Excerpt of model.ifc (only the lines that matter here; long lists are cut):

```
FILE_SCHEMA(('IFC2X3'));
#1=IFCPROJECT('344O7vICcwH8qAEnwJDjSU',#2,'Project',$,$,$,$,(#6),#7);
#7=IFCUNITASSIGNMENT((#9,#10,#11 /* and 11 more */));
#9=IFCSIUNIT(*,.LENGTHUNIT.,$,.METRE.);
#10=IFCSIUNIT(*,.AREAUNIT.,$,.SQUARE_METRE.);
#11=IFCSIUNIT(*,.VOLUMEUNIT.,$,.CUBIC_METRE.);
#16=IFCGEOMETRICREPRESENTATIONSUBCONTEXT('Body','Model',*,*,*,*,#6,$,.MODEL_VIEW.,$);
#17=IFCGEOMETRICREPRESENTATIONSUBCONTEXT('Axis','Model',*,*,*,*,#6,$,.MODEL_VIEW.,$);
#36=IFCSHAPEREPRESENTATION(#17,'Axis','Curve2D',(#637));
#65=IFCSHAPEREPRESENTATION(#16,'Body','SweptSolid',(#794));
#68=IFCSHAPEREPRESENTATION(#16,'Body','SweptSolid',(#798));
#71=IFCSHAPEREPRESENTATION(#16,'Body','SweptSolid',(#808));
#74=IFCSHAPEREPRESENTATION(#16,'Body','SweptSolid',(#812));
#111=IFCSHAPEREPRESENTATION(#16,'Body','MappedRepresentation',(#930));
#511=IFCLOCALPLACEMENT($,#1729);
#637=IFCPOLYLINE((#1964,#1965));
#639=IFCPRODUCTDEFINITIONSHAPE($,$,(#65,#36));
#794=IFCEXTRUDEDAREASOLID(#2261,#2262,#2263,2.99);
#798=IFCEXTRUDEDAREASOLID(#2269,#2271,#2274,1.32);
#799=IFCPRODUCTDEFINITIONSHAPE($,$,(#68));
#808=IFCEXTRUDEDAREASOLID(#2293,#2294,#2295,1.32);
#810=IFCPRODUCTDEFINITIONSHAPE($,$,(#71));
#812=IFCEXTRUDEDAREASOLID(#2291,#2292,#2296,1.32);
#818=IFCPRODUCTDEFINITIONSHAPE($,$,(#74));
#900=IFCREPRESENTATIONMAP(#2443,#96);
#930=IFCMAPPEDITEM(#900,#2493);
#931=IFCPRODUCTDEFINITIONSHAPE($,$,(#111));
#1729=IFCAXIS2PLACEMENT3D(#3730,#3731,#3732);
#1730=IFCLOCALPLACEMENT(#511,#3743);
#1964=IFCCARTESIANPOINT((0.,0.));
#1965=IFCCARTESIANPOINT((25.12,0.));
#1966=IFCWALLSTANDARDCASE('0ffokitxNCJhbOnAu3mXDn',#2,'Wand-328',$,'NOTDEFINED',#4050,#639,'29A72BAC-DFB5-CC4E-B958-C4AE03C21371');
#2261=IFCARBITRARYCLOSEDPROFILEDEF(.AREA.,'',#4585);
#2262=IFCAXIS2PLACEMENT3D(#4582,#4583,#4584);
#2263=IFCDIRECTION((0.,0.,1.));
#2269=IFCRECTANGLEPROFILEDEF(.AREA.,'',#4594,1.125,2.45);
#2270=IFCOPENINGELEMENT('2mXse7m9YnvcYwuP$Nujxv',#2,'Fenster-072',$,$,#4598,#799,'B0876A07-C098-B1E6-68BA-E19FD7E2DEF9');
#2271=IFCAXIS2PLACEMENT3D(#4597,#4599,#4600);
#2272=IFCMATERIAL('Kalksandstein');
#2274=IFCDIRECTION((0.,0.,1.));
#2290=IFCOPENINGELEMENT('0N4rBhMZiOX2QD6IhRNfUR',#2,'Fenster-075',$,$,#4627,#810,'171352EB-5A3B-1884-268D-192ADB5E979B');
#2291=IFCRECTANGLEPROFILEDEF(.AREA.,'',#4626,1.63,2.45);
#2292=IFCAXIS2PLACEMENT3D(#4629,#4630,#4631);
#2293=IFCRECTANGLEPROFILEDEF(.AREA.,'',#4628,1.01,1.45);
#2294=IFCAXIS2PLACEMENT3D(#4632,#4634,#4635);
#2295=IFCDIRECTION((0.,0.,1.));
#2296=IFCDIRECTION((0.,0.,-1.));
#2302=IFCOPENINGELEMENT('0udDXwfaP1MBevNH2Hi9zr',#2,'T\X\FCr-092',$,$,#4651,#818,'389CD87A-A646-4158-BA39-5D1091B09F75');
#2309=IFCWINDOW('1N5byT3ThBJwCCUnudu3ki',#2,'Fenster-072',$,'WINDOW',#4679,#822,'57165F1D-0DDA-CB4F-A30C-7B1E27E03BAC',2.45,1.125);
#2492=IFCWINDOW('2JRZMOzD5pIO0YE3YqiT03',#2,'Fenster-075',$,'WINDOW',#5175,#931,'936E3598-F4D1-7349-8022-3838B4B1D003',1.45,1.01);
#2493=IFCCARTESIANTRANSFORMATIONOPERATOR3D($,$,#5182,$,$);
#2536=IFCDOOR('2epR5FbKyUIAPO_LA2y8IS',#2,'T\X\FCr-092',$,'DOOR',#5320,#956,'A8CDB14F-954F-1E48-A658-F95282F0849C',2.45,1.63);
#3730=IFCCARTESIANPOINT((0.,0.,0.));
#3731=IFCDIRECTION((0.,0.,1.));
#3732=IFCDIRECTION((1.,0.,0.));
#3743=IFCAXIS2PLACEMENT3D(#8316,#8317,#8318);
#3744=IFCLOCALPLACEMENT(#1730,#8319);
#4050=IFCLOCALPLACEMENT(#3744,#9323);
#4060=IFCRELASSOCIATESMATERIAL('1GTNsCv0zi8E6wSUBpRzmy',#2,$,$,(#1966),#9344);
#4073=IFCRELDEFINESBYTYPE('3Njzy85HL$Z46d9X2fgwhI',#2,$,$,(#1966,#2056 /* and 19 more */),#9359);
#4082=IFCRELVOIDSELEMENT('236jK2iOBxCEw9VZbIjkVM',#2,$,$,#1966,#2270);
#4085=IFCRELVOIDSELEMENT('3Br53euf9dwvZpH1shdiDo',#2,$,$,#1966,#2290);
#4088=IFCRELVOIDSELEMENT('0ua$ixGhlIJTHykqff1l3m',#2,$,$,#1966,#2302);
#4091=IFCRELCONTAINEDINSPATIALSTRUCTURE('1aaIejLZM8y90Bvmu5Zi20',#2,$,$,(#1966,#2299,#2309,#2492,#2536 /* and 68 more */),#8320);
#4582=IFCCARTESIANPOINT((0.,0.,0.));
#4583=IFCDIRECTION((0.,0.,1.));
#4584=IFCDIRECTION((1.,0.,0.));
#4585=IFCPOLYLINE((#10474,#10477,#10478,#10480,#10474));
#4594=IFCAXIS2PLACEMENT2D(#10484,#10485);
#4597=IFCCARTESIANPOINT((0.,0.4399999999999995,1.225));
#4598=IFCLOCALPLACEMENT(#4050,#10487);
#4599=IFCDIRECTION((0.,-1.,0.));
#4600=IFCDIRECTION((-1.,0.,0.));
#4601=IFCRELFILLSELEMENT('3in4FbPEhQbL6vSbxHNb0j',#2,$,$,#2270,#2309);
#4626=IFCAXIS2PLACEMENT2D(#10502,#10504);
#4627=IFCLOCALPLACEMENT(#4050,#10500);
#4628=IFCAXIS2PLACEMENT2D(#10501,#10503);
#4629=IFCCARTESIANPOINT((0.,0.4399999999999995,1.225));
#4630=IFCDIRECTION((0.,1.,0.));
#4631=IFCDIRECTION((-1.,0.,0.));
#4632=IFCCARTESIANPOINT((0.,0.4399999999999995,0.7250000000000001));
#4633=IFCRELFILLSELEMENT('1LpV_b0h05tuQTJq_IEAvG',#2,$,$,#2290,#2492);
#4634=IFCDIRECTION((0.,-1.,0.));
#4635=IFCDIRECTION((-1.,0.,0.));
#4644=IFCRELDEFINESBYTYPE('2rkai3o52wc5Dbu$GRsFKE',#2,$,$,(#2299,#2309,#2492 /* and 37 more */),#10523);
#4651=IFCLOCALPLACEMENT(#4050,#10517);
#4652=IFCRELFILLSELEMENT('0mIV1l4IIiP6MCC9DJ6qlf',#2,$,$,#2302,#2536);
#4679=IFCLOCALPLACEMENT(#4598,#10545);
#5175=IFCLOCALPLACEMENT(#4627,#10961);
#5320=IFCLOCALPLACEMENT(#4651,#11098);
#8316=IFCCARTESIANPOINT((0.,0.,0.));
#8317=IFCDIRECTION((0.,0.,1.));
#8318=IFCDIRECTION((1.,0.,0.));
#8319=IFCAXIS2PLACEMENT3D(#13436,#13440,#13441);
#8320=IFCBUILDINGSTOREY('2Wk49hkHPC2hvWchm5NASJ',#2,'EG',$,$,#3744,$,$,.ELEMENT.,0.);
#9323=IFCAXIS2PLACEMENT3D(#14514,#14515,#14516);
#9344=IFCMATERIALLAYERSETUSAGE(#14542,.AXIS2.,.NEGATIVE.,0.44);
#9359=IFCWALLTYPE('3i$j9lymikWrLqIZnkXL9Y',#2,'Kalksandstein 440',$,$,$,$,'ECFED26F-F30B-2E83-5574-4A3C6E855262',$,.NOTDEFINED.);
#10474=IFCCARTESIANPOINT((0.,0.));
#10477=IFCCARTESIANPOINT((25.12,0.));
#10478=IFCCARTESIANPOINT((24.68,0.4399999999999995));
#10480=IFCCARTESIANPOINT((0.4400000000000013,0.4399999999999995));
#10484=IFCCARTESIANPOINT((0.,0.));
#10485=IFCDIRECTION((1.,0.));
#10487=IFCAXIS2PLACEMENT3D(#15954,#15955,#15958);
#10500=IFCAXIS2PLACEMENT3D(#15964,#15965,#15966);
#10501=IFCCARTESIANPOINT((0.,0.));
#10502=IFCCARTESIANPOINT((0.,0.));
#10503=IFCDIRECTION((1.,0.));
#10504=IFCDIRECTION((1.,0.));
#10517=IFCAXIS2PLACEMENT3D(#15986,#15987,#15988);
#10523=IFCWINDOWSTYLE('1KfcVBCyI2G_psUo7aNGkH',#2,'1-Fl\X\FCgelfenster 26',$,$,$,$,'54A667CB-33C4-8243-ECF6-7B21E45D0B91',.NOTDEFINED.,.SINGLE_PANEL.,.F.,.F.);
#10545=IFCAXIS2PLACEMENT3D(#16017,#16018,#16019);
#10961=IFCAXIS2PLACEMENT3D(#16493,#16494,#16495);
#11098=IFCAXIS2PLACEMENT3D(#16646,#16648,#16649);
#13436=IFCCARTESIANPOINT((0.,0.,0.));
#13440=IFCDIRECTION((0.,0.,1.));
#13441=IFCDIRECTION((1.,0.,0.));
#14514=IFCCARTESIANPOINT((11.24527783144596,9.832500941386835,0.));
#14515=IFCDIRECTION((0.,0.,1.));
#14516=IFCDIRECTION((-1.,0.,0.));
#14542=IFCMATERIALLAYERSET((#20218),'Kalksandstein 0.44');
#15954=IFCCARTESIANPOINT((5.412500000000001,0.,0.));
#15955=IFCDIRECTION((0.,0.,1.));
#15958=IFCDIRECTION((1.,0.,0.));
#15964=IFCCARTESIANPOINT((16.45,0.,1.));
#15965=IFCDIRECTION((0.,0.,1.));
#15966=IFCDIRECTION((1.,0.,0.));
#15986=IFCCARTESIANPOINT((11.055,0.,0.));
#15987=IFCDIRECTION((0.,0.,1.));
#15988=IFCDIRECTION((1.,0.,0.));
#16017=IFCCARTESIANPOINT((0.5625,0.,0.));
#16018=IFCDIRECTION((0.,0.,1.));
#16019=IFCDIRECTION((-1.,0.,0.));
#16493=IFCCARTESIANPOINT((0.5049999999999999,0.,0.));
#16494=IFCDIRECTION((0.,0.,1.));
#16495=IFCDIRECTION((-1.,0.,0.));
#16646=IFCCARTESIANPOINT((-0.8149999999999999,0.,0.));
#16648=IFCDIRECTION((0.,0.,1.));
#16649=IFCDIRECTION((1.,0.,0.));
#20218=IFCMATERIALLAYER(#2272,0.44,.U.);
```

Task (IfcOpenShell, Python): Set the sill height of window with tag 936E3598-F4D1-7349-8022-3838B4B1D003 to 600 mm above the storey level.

```python
import numpy as np
import ifcopenshell
import ifcopenshell.api.geometry
import ifcopenshell.geom
import ifcopenshell.util.element
import ifcopenshell.util.placement
import ifcopenshell.util.shape
import ifcopenshell.util.unit

model = ifcopenshell.open("model.ifc")
unit_scale = ifcopenshell.util.unit.calculate_unit_scale(model)

window = model.by_guid("2JRZMOzD5pIO0YE3YqiT03")
opening = window.FillsVoids[0].RelatingOpeningElement
storey = ifcopenshell.util.element.get_container(window, ifc_class="IfcBuildingStorey")
level = ifcopenshell.util.placement.get_local_placement(storey.ObjectPlacement)[2, 3]

# The opening's origin need not be at the sill, so measure its lowest point.
shape = ifcopenshell.geom.create_shape(ifcopenshell.geom.settings(), opening)
bottom = ifcopenshell.util.shape.get_shape_bottom_elevation(shape, shape.geometry) / unit_scale
dz = level + 0.6 / unit_scale - bottom

shift = np.array([0.0, 0.0, dz])
# The window is placed relative to its opening, so it follows when the opening moves.
matrix = ifcopenshell.util.placement.get_local_placement(opening.ObjectPlacement)
matrix[:3, 3] += shift
ifcopenshell.api.geometry.edit_object_placement(
    model, product=opening, matrix=matrix, is_si=False, should_transform_children=True
)

print(f"moved by {dz * unit_scale:+.3f} m")

model.write("model_updated.ifc")
```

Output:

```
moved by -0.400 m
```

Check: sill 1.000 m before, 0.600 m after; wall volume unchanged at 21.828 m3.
